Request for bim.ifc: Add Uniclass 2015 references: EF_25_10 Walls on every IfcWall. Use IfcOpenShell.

First a look at what the model holds.

```python
import ifcopenshell

model = ifcopenshell.open("bim.ifc")
print(model.schema)
print("classifications:", [c.Name for c in model.by_type("IfcClassification")])
for ifc_class in ("IfcDoor", "IfcRoof", "IfcStair", "IfcWall", "IfcWindow"):
    print(ifc_class, len(model.by_type(ifc_class)))
```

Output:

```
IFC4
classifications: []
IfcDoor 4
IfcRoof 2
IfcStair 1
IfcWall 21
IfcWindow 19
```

```python
import ifcopenshell
import ifcopenshell.api.classification

model = ifcopenshell.open("bim.ifc")

system = ifcopenshell.api.classification.add_classification(model, classification="Uniclass 2015")

codes = {
    "IfcWall": ("EF_25_10", "Walls"),
}
for ifc_class, (code, name) in codes.items():
    products = model.by_type(ifc_class)
    ifcopenshell.api.classification.add_reference(
        model, products=products, classification=system, identification=code, name=name
    )
    print(code, len(products))

model.write("bim_updated.ifc")
```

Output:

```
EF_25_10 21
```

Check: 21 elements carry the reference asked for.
